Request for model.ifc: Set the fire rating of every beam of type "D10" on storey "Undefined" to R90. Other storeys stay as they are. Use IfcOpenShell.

First a look at what the model holds.

```python
import ifcopenshell
import ifcopenshell.util.element

model = ifcopenshell.open("model.ifc")
print(model.schema)
storey = next(s for s in model.by_type("IfcBuildingStorey") if s.Name == "Undefined")
beams = [e for e in ifcopenshell.util.element.get_decomposition(storey) if e.is_a("IfcBeam")]
seen = {}
for e in beams:
    element_type = ifcopenshell.util.element.get_type(e)
    key = (element_type.Name if element_type != e and element_type else None, ifcopenshell.util.element.get_pset(e, "Pset_BeamCommon", "FireRating"))
    seen[key] = seen.get(key, 0) + 1
for (name, value), count in sorted(seen.items(), key=str):
    print(count, "x", name, "|", value)
```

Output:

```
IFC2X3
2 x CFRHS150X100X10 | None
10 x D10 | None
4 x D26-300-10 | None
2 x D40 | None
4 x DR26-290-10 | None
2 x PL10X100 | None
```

```python
import ifcopenshell
import ifcopenshell.api.pset
import ifcopenshell.util.element

model = ifcopenshell.open("model.ifc")

storey = next(s for s in model.by_type("IfcBuildingStorey") if s.Name == "Undefined")
beams = [e for e in ifcopenshell.util.element.get_decomposition(storey) if e.is_a("IfcBeam")]

count = 0
for e in beams:
    element_type = ifcopenshell.util.element.get_type(e)
    if element_type in (None, e) or element_type.Name != "D10":
        continue
    found = ifcopenshell.util.element.get_pset(e, "Pset_BeamCommon", should_inherit=False)
    if found:
        pset = model.by_id(found["id"])
        if len(ifcopenshell.util.element.get_elements_by_pset(pset)) > 1:
            pset = ifcopenshell.api.pset.unshare_pset(model, products=[e], pset=pset)[0]
    else:
        pset = ifcopenshell.api.pset.add_pset(model, product=e, name="Pset_BeamCommon")
    ifcopenshell.api.pset.edit_pset(model, pset=pset, properties={"FireRating": "R90"})
    count += 1

print(count, "beams updated")

model.write("model_v2.ifc")
```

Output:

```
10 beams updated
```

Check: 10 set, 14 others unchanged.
